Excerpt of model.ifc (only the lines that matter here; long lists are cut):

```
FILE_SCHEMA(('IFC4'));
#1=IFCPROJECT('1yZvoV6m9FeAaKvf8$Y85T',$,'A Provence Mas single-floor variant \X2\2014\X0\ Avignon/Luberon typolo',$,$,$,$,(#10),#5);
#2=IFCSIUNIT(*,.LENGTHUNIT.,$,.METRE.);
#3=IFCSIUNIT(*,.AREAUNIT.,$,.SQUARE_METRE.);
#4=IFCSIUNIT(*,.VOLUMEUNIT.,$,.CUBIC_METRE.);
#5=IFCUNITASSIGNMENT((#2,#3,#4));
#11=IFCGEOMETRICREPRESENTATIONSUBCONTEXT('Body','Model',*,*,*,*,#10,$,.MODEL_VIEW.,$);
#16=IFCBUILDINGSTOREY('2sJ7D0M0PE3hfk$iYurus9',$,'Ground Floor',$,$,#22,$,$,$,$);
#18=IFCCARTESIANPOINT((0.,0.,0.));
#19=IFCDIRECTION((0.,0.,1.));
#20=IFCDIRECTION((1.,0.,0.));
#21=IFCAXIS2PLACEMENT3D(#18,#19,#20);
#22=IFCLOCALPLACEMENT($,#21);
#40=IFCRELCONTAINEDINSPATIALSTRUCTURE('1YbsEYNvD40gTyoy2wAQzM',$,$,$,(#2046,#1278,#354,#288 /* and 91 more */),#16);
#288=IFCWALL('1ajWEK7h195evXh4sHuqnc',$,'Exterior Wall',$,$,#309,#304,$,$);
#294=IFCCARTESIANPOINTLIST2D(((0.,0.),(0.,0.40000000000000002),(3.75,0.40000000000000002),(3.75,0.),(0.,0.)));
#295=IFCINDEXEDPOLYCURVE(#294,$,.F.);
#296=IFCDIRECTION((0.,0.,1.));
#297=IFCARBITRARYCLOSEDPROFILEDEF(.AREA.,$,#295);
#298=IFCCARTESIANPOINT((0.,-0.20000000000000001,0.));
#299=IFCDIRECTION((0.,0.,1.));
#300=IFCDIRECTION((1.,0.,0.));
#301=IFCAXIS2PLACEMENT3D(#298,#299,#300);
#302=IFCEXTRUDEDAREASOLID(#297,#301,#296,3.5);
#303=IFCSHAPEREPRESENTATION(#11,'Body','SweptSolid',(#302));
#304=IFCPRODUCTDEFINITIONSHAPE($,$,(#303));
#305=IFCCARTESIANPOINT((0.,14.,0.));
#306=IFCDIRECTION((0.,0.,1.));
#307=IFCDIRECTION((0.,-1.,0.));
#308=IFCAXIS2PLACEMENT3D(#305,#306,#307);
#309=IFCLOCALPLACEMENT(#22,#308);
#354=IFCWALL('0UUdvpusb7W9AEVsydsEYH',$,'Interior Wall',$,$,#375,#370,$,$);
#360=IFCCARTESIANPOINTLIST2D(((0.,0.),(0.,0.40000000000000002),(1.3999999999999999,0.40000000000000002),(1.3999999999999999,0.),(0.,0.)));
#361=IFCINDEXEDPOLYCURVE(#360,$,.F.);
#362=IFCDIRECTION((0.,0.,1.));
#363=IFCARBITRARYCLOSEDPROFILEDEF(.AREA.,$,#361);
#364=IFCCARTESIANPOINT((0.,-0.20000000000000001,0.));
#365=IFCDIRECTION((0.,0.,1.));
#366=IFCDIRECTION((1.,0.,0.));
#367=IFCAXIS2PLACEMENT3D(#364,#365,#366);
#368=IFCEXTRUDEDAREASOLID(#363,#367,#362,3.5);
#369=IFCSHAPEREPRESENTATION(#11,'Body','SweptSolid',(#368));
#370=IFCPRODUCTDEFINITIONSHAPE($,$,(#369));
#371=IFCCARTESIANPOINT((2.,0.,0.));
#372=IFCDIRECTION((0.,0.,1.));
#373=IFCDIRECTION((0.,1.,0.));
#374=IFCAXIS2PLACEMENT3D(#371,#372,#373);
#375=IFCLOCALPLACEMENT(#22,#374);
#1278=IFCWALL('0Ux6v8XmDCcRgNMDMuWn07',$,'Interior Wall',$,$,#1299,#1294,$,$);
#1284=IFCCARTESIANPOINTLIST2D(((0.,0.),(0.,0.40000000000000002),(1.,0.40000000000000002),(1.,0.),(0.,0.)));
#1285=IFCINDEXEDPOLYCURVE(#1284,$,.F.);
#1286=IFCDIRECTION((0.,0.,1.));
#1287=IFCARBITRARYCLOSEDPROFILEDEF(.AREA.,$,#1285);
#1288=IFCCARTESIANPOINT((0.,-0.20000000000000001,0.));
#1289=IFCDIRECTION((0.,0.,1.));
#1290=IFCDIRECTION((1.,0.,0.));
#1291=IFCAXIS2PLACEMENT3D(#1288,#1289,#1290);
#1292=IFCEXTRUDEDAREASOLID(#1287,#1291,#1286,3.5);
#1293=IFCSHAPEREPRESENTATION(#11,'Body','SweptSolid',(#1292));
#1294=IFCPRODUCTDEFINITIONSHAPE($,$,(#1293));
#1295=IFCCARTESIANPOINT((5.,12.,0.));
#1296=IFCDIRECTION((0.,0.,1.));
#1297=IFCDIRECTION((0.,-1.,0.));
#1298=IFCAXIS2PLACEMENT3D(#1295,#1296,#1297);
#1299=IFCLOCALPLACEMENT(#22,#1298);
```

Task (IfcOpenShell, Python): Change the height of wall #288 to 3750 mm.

```python
import ifcopenshell
import ifcopenshell.geom
import ifcopenshell.util.representation
import ifcopenshell.util.shape
import ifcopenshell.util.unit

model = ifcopenshell.open("model.ifc")
unit_scale = ifcopenshell.util.unit.calculate_unit_scale(model)
settings = ifcopenshell.geom.settings()


def volume(element):
    """Net volume in cubic metres, openings subtracted."""
    shape = ifcopenshell.geom.create_shape(settings, element)
    return ifcopenshell.util.shape.get_volume(shape.geometry)


wall = model.by_guid("1ajWEK7h195evXh4sHuqnc")
before = volume(wall)

body = ifcopenshell.util.representation.get_representation(wall, "Model", "Body")
solid = body.Items[0]
old_height = solid.Depth
solid.Depth = 3.75 / unit_scale
after = volume(wall)

print(f"height {old_height:g} -> {solid.Depth:g}, volume {before:.3f} -> {after:.3f} m3")

model.write("model_v2.ifc")
```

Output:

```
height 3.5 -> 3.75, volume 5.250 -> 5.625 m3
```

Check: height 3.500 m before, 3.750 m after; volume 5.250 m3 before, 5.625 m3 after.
